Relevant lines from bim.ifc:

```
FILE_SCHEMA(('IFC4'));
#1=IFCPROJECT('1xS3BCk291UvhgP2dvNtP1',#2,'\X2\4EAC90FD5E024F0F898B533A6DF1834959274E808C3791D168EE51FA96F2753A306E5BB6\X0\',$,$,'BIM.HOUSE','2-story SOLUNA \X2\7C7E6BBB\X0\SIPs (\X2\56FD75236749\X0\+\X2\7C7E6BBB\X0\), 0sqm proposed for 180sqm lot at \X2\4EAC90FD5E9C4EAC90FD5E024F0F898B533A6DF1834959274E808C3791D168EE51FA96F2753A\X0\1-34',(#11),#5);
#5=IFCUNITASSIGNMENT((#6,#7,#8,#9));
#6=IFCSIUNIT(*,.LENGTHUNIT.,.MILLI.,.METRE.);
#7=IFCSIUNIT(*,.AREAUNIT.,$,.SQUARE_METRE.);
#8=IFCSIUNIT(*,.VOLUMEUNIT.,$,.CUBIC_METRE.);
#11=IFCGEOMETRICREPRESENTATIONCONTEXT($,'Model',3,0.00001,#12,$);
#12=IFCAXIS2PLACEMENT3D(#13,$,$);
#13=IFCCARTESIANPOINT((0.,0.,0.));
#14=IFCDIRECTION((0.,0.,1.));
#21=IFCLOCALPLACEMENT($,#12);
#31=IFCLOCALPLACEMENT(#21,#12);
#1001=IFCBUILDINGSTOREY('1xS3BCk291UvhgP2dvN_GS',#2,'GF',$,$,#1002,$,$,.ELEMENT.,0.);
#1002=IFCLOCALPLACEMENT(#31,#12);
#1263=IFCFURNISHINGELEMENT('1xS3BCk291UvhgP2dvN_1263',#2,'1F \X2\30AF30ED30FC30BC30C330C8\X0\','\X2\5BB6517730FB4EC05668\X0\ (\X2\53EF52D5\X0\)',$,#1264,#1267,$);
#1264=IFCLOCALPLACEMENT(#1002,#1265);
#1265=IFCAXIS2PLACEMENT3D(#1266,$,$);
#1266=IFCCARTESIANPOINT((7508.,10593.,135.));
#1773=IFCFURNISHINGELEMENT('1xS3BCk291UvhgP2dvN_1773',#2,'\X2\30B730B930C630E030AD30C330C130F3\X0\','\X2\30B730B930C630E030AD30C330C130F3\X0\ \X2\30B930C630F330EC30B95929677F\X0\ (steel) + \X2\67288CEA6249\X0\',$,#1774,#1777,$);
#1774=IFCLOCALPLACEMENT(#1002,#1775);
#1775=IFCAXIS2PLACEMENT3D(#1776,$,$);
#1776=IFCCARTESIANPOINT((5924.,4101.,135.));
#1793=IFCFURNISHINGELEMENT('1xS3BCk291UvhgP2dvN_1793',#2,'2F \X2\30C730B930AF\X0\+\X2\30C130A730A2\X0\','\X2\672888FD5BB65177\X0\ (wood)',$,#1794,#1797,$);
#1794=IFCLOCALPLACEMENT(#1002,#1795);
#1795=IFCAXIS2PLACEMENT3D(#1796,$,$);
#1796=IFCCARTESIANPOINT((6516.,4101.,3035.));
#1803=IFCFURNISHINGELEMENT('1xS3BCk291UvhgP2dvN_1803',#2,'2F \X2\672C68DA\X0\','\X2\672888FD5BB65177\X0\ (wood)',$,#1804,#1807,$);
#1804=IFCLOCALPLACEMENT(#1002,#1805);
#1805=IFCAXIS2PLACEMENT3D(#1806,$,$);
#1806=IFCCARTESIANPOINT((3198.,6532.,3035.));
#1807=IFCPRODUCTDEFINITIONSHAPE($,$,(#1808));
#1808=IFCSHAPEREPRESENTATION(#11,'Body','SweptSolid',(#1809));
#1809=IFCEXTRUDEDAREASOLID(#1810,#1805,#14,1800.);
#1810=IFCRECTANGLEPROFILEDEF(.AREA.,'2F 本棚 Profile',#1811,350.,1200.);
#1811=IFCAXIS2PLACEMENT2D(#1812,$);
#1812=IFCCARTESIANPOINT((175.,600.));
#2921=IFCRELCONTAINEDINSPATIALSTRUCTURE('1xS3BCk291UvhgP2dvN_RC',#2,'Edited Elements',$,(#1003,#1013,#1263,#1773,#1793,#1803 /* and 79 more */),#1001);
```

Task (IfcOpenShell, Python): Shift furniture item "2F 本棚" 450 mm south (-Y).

```python
import ifcopenshell
import ifcopenshell.api.geometry
import ifcopenshell.util.placement

model = ifcopenshell.open("bim.ifc")

item = model.by_guid("1xS3BCk291UvhgP2dvN_1803")
matrix = ifcopenshell.util.placement.get_local_placement(item.ObjectPlacement)
matrix[1, 3] -= 450.0
ifcopenshell.api.geometry.edit_object_placement(model, product=item, matrix=matrix, is_si=False)

print(ifcopenshell.util.placement.get_local_placement(item.ObjectPlacement).round(3) + 0.0)

model.write("bim_updated.ifc")
```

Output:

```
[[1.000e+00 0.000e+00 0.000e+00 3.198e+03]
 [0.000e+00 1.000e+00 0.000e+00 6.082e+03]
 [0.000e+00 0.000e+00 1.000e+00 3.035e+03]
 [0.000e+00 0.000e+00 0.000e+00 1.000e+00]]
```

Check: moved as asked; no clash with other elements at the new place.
